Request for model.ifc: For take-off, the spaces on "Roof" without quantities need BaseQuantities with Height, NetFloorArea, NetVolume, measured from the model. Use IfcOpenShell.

First a look at what the model holds.

```python
import ifcopenshell
import ifcopenshell.util.element
import ifcopenshell.util.unit

model = ifcopenshell.open("model.ifc")
print(model.schema)
for unit_type in ("LENGTHUNIT", "AREAUNIT", "VOLUMEUNIT"):
    print(unit_type, ifcopenshell.util.unit.calculate_unit_scale(model, unit_type))
storey = next(s for s in model.by_type("IfcBuildingStorey") if s.Name == "Roof")
spaces = [e for e in ifcopenshell.util.element.get_decomposition(storey) if e.is_a("IfcSpace")]
for e in sorted(spaces, key=lambda e: e.id()):
    print(e.id(), e.is_a(), e.Name, list(ifcopenshell.util.element.get_psets(e, qtos_only=True)), sep=" | ")
```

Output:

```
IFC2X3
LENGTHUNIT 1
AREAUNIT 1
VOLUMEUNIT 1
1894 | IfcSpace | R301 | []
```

```python
import ifcopenshell
import ifcopenshell.api.pset
import ifcopenshell.geom
import ifcopenshell.util.element
import ifcopenshell.util.shape
import ifcopenshell.util.unit

model = ifcopenshell.open("model.ifc")
unit_scale = ifcopenshell.util.unit.calculate_unit_scale(model)
area_scale = ifcopenshell.util.unit.calculate_unit_scale(model, "AREAUNIT")
volume_scale = ifcopenshell.util.unit.calculate_unit_scale(model, "VOLUMEUNIT")
settings = ifcopenshell.geom.settings()

storey = next(s for s in model.by_type("IfcBuildingStorey") if s.Name == "Roof")
spaces = [e for e in ifcopenshell.util.element.get_decomposition(storey) if e.is_a("IfcSpace")]

for e in sorted(spaces, key=lambda e: e.id()):
    if ifcopenshell.util.element.get_psets(e, qtos_only=True, should_inherit=False):
        continue
    # Geometry comes back in metres, in the element's own axes.
    shape = ifcopenshell.geom.create_shape(settings, e)
    values = {
        "Height": ifcopenshell.util.shape.get_z(shape.geometry) / unit_scale,
        "NetFloorArea": ifcopenshell.util.shape.get_footprint_area(shape.geometry) / area_scale,
        "NetVolume": ifcopenshell.util.shape.get_volume(shape.geometry) / volume_scale,
    }
    qto = ifcopenshell.api.pset.add_qto(model, product=e, name="BaseQuantities")
    ifcopenshell.api.pset.edit_qto(model, qto=qto, properties=values)
    print(e.id(), {k: round(v, 3) for k, v in values.items()})

model.write("model_updated.ifc")
```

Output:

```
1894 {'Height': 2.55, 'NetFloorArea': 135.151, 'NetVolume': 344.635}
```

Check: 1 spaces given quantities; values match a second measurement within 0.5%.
